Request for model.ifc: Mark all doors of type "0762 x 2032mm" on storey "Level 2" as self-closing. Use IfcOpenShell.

First a look at what the model holds.

```python
import ifcopenshell
import ifcopenshell.util.element

model = ifcopenshell.open("model.ifc")
print(model.schema)
storey = next(s for s in model.by_type("IfcBuildingStorey") if s.Name == "Level 2")
doors = [e for e in ifcopenshell.util.element.get_decomposition(storey) if e.is_a("IfcDoor")]
seen = {}
for e in doors:
    element_type = ifcopenshell.util.element.get_type(e)
    key = (element_type.Name if element_type != e and element_type else None, ifcopenshell.util.element.get_pset(e, "Pset_DoorCommon", "SelfClosing"))
    seen[key] = seen.get(key, 0) + 1
for (name, value), count in sorted(seen.items(), key=str):
    print(count, "x", name, "|", value)
```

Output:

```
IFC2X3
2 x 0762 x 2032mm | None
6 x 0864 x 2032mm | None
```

```python
import ifcopenshell
import ifcopenshell.api.pset
import ifcopenshell.util.element

model = ifcopenshell.open("model.ifc")

storey = next(s for s in model.by_type("IfcBuildingStorey") if s.Name == "Level 2")
doors = [e for e in ifcopenshell.util.element.get_decomposition(storey) if e.is_a("IfcDoor")]

count = 0
for e in doors:
    element_type = ifcopenshell.util.element.get_type(e)
    if element_type in (None, e) or element_type.Name != "0762 x 2032mm":
        continue
    # add_pset returns the element's existing set when there is one.
    pset = ifcopenshell.api.pset.add_pset(model, product=e, name="Pset_DoorCommon")
    ifcopenshell.api.pset.edit_pset(model, pset=pset, properties={"SelfClosing": True})
    count += 1

print(count, "doors updated")

model.write("model_v2.ifc")
```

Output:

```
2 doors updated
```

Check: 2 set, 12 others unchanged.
